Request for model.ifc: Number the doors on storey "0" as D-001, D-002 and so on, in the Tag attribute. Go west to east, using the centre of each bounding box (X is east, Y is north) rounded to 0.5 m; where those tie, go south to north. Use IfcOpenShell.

First a look at what the model holds.

```python
import ifcopenshell
import ifcopenshell.util.element
import ifcopenshell.util.placement

model = ifcopenshell.open("model.ifc")
print(model.schema)
storey = next(s for s in model.by_type("IfcBuildingStorey") if s.Name == "0")
doors = [e for e in ifcopenshell.util.element.get_decomposition(storey) if e.is_a("IfcDoor")]
for e in sorted(doors, key=lambda e: e.id()):
    origin = ifcopenshell.util.placement.get_local_placement(e.ObjectPlacement)[:3, 3]
    print(e.id(), e.Tag, e.Name, origin.round(2) + 0.0, sep=" | ")
```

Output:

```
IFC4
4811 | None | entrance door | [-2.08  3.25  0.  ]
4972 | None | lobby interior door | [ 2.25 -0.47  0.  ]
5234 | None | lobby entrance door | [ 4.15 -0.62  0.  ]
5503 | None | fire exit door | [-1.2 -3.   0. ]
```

```python
import ifcopenshell
import ifcopenshell.geom
import ifcopenshell.util.element
import ifcopenshell.util.shape

model = ifcopenshell.open("model.ifc")
settings = ifcopenshell.geom.settings()
settings.set("use-world-coords", True)


def centre(element):
    shape = ifcopenshell.geom.create_shape(settings, element)
    return ifcopenshell.util.shape.get_bbox_centroid(shape.geometry)


storey = next(s for s in model.by_type("IfcBuildingStorey") if s.Name == "0")
doors = [e for e in ifcopenshell.util.element.get_decomposition(storey) if e.is_a("IfcDoor")]

# Insertion points can sit at a corner or the storey origin, so sort by the geometry (in metres).
centres = {e: centre(e) for e in doors}
doors.sort(key=lambda e: (round(centres[e][0] / 0.5), centres[e][1]))

for i, e in enumerate(doors, start=1):
    number = f"D-0{i:02d}"
    e.Tag = number
    print(e.id(), number)

model.write("model_updated.ifc")
```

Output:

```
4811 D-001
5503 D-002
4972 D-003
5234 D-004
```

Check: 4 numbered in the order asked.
